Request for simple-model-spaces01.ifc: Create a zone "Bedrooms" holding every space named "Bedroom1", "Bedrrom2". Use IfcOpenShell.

First a look at what the model holds.

```python
import ifcopenshell

model = ifcopenshell.open("simple-model-spaces01.ifc")
print(model.schema)
seen = {}
for space in model.by_type("IfcSpace"):
    seen[space.LongName] = seen.get(space.LongName, 0) + 1
for name, count in sorted(seen.items(), key=str):
    print(count, "x", name)
print("zones:", [z.Name for z in model.by_type("IfcZone")][:20])
```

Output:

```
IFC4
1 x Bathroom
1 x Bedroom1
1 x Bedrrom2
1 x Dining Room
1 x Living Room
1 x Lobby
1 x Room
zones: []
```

```python
import ifcopenshell
import ifcopenshell.api.group
import ifcopenshell.api.root

model = ifcopenshell.open("simple-model-spaces01.ifc")

names = {"Bedroom1", "Bedrrom2"}
spaces = [s for s in model.by_type("IfcSpace") if s.LongName in names]

zone = ifcopenshell.api.root.create_entity(model, ifc_class="IfcZone", name="Bedrooms")
ifcopenshell.api.group.assign_group(model, products=spaces, group=zone)
print(len(spaces), "spaces in", zone.Name)

model.write("simple-model-spaces01_edited.ifc")
```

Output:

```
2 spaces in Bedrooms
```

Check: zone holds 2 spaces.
